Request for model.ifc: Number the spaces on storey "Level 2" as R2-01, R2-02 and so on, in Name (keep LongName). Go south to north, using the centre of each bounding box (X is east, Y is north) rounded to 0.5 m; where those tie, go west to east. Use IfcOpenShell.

First a look at what the model holds.

```python
import ifcopenshell
import ifcopenshell.util.element
import ifcopenshell.util.placement

model = ifcopenshell.open("model.ifc")
print(model.schema)
storey = next(s for s in model.by_type("IfcBuildingStorey") if s.Name == "Level 2")
spaces = [e for e in ifcopenshell.util.element.get_decomposition(storey) if e.is_a("IfcSpace")]
for e in sorted(spaces, key=lambda e: e.id()):
    origin = ifcopenshell.util.placement.get_local_placement(e.ObjectPlacement)[:3, 3]
    print(e.id(), e.Name, e.LongName, origin.round(2) + 0.0, sep=" | ")
```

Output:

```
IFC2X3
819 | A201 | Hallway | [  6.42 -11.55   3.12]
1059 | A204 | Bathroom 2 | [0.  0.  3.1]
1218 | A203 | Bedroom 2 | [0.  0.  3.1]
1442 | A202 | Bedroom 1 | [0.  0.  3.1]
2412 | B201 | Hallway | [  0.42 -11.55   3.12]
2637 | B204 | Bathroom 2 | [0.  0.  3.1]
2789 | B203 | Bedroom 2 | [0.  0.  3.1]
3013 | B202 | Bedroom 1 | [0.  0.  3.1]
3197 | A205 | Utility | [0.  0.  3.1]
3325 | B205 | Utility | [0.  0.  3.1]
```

```python
import ifcopenshell
import ifcopenshell.geom
import ifcopenshell.util.element
import ifcopenshell.util.shape

model = ifcopenshell.open("model.ifc")
settings = ifcopenshell.geom.settings()
settings.set("use-world-coords", True)


def centre(element):
    shape = ifcopenshell.geom.create_shape(settings, element)
    return ifcopenshell.util.shape.get_bbox_centroid(shape.geometry)


storey = next(s for s in model.by_type("IfcBuildingStorey") if s.Name == "Level 2")
spaces = [e for e in ifcopenshell.util.element.get_decomposition(storey) if e.is_a("IfcSpace")]

# Insertion points can sit at a corner or the storey origin, so sort by the geometry (in metres).
centres = {e: centre(e) for e in spaces}
spaces.sort(key=lambda e: (round(centres[e][1] / 0.5), centres[e][0]))

for i, e in enumerate(spaces, start=1):
    number = f"R2-{i:02d}"
    e.Name = number
    print(e.id(), number)

model.write("model-out.ifc")
```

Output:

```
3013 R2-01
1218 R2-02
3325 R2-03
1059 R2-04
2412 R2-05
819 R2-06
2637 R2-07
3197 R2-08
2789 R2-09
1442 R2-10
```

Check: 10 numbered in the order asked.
